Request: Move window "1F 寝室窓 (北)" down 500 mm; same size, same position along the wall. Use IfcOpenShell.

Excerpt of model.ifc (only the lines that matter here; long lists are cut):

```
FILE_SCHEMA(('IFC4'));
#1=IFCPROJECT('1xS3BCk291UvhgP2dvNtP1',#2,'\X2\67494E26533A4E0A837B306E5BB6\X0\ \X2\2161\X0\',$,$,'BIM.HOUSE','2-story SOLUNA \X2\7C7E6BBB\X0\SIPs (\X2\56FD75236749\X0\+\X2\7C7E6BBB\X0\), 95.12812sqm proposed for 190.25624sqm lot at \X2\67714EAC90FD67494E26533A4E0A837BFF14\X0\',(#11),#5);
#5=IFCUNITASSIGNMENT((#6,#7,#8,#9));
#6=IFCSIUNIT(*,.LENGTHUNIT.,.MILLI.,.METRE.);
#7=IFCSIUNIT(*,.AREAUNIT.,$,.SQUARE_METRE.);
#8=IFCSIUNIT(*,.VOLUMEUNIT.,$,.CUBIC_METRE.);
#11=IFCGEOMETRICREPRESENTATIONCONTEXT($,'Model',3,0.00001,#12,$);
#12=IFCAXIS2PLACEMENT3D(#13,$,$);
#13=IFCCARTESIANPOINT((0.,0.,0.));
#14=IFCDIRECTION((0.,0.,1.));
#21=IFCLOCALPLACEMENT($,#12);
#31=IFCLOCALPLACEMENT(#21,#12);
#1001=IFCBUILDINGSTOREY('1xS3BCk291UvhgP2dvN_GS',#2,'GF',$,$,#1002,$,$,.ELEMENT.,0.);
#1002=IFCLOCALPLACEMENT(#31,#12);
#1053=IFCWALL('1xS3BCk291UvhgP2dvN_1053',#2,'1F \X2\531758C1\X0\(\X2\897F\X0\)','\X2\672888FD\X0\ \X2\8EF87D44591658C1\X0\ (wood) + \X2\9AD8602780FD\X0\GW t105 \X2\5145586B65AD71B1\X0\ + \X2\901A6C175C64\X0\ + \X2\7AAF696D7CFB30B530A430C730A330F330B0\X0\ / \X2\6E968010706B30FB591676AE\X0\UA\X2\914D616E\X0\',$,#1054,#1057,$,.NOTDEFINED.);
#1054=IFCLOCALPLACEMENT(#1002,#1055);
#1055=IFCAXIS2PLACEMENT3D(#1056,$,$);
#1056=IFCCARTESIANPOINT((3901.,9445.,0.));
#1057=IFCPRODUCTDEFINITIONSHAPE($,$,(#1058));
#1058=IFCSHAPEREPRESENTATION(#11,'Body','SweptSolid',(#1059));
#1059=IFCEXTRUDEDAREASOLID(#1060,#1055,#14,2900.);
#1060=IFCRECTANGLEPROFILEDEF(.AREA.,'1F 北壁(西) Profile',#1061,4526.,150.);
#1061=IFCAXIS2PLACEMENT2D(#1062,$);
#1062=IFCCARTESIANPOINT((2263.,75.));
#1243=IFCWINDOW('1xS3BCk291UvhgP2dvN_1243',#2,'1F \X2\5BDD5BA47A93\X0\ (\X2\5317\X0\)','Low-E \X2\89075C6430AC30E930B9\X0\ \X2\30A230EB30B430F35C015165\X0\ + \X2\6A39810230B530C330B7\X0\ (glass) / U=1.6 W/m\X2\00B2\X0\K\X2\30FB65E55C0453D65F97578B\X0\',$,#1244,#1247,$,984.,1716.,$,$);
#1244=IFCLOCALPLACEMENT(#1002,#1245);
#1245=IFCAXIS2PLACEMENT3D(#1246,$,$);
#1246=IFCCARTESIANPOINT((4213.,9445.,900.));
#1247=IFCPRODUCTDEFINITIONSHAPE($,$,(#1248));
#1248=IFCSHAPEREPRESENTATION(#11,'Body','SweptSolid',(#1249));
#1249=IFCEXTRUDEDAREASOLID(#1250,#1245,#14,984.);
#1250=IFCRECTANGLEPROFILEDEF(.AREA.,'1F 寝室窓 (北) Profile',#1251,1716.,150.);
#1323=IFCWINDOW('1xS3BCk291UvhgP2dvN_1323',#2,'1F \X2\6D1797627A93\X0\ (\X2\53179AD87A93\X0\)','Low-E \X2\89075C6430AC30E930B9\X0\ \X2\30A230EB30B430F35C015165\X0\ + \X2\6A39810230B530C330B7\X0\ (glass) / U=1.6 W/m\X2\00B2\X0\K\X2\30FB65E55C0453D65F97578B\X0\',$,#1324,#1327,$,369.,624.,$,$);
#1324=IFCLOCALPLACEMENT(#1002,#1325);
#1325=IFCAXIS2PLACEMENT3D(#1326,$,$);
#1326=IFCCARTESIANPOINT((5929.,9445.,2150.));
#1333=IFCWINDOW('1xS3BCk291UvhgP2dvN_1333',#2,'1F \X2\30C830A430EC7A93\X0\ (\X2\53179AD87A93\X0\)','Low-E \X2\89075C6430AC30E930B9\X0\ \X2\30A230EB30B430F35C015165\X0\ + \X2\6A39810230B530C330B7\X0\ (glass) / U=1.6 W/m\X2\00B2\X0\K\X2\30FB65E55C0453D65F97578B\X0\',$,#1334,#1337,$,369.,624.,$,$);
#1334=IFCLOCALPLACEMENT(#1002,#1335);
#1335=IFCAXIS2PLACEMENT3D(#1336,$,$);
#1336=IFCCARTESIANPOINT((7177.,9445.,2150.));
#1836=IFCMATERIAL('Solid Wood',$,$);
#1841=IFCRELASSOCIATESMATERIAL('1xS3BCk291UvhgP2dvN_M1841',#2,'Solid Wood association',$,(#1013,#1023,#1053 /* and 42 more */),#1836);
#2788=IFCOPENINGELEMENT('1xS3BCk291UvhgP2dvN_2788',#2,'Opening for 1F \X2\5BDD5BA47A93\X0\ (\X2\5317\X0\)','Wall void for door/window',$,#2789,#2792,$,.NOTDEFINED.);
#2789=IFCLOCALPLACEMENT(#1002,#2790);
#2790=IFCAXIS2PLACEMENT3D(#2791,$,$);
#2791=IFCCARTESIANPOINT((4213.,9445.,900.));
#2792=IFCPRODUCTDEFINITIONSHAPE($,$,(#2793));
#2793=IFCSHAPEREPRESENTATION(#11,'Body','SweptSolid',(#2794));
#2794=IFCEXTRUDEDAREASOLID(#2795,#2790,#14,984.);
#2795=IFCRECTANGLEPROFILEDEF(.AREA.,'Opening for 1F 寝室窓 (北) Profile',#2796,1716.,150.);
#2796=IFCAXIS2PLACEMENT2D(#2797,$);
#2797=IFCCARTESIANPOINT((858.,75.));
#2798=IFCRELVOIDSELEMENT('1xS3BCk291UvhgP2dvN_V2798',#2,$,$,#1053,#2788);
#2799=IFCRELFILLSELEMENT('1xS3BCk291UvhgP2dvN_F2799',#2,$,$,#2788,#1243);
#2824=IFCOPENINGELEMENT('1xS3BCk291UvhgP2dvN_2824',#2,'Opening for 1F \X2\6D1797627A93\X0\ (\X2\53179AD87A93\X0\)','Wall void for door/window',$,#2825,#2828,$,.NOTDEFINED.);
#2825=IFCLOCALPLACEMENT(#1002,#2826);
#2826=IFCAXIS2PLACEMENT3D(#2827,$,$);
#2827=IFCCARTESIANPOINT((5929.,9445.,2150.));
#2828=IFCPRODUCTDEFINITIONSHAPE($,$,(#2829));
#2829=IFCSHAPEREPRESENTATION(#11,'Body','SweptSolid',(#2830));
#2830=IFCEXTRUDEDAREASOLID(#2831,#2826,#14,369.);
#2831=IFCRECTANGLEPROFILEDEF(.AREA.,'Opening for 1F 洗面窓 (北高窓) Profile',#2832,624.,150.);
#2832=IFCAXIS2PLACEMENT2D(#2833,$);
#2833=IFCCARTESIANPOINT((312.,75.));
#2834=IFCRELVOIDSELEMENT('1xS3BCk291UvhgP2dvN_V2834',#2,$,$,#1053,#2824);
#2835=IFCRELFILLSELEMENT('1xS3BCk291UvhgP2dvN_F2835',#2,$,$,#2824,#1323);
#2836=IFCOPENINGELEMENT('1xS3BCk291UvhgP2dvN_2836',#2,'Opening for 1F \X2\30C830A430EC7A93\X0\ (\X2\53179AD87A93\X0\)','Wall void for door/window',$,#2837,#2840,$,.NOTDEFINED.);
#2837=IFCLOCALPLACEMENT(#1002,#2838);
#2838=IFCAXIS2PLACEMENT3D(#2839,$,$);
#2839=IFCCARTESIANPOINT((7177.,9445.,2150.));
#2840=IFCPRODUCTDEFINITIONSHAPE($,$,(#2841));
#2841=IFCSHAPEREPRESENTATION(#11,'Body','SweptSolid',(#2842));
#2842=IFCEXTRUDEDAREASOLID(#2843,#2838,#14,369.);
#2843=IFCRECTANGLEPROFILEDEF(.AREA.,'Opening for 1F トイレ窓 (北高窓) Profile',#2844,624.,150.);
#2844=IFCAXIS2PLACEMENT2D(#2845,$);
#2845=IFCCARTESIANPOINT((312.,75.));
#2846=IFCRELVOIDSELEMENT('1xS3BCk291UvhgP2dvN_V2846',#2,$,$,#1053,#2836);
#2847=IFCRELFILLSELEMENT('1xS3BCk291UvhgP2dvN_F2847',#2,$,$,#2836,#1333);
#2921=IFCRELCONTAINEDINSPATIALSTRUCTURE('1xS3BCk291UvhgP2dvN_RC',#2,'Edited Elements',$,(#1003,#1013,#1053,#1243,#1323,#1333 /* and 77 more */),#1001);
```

```python
import numpy as np
import ifcopenshell
import ifcopenshell.api.geometry
import ifcopenshell.util.placement
import ifcopenshell.util.unit

model = ifcopenshell.open("model.ifc")
unit_scale = ifcopenshell.util.unit.calculate_unit_scale(model)

window = model.by_guid("1xS3BCk291UvhgP2dvN_1243")
opening = window.FillsVoids[0].RelatingOpeningElement
dz = -500.0

shift = np.array([0.0, 0.0, dz])
# The window is not placed relative to its opening, so move both.
for product in (opening, window):
    matrix = ifcopenshell.util.placement.get_local_placement(product.ObjectPlacement)
    matrix[:3, 3] += shift
    ifcopenshell.api.geometry.edit_object_placement(model, product=product, matrix=matrix, is_si=False)

print(f"moved by {dz * unit_scale:+.3f} m")

model.write("model_edited.ifc")
```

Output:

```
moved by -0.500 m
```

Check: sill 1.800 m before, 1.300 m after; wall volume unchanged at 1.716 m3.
